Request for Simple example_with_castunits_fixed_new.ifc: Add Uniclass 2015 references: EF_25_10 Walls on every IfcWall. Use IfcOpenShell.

First a look at what the model holds.

```python
import ifcopenshell

model = ifcopenshell.open("Simple example_with_castunits_fixed_new.ifc")
print(model.schema)
print("classifications:", [c.Name for c in model.by_type("IfcClassification")])
for ifc_class in ("IfcDoor", "IfcRoof", "IfcStair", "IfcWall", "IfcWindow"):
    print(ifc_class, len(model.by_type(ifc_class)))
```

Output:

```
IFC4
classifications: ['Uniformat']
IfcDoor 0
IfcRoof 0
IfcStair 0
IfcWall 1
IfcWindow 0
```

```python
import ifcopenshell
import ifcopenshell.api.classification

model = ifcopenshell.open("Simple example_with_castunits_fixed_new.ifc")

system = ifcopenshell.api.classification.add_classification(model, classification="Uniclass 2015")

codes = {
    "IfcWall": ("EF_25_10", "Walls"),
}
for ifc_class, (code, name) in codes.items():
    products = model.by_type(ifc_class)
    ifcopenshell.api.classification.add_reference(
        model, products=products, classification=system, identification=code, name=name
    )
    print(code, len(products))

model.write("Simple example_with_castunits_fixed_new_v2.ifc")
```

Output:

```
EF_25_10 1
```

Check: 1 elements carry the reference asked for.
